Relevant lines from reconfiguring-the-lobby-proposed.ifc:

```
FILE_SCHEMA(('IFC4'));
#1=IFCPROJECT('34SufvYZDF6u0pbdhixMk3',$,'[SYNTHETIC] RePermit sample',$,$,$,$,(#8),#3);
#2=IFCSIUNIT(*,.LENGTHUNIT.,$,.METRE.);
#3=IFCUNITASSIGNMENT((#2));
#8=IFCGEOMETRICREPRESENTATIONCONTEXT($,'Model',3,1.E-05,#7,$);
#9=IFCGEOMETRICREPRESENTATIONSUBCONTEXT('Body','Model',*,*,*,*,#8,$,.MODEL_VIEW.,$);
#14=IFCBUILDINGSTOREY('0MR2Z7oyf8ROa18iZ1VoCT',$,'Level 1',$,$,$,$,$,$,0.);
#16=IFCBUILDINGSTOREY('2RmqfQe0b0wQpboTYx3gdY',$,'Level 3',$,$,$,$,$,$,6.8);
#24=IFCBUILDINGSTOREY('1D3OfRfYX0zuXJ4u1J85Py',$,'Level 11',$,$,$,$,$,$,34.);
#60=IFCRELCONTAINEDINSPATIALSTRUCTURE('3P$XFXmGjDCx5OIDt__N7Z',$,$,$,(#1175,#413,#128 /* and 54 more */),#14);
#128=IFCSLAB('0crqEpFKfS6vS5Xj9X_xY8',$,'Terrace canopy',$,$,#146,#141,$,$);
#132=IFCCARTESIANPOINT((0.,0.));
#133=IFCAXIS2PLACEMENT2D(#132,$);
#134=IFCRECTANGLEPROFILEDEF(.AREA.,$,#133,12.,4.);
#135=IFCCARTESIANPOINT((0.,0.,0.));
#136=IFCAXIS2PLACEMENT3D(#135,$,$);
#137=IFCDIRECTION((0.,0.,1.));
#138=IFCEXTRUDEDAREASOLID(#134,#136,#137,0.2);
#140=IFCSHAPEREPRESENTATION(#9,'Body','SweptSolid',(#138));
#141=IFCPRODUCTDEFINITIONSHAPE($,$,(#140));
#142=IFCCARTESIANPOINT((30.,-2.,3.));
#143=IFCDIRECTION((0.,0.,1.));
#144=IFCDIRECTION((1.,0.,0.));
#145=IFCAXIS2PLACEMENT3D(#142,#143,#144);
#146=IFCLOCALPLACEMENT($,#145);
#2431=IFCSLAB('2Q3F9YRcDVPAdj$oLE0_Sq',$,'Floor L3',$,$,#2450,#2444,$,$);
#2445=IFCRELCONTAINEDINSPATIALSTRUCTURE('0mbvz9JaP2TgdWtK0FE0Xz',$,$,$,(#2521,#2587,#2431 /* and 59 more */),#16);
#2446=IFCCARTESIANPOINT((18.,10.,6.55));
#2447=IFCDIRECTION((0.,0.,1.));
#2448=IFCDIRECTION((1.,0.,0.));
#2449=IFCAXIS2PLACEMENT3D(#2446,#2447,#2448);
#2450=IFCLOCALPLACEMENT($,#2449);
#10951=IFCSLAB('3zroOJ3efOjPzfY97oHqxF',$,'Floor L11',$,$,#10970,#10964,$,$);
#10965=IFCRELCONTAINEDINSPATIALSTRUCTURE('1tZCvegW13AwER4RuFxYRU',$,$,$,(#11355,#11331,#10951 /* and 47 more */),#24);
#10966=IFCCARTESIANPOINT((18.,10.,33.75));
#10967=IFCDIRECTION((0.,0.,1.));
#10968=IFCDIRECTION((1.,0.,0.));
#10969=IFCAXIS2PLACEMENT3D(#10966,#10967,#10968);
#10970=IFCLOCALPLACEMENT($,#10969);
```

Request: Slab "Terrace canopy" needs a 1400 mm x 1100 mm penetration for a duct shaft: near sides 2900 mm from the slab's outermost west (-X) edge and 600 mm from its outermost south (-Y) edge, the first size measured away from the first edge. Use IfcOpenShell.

```python
import numpy as np
import ifcopenshell
import ifcopenshell.api.feature
import ifcopenshell.api.geometry
import ifcopenshell.api.root
import ifcopenshell.geom
import ifcopenshell.util.placement
import ifcopenshell.util.representation
import ifcopenshell.util.shape
import ifcopenshell.util.unit

model = ifcopenshell.open("reconfiguring-the-lobby-proposed.ifc")
unit_scale = ifcopenshell.util.unit.calculate_unit_scale(model)
settings = ifcopenshell.geom.settings()


def volume(element):
    """Net volume in cubic metres, openings subtracted."""
    shape = ifcopenshell.geom.create_shape(settings, element)
    return ifcopenshell.util.shape.get_volume(shape.geometry)


slab = model.by_guid("0crqEpFKfS6vS5Xj9X_xY8")
before = volume(slab)

# Extent in the slab's own axes, in metres. The edges named are its -X and -Y sides.
slab_shape = ifcopenshell.geom.create_shape(settings, slab)
vertices = ifcopenshell.util.shape.get_vertices(slab_shape.geometry)
x_min, y_min, bottom = vertices.min(axis=0)
top = vertices[:, 2].max()

opening = ifcopenshell.api.root.create_entity(model, ifc_class="IfcOpeningElement", name="Duct shaft opening", predefined_type="OPENING")
context = ifcopenshell.util.representation.get_context(model, "Model", "Body", "MODEL_VIEW")
width, depth = 1.4, 1.1
outline = [(0.0, 0.0), (width, 0.0), (width, depth), (0.0, depth), (0.0, 0.0)]
# Overshoot both faces by 50 mm so the cut is clean.
shape = ifcopenshell.api.geometry.add_slab_representation(
    model, context=context, depth=top - bottom + 0.1, polyline=outline
)
ifcopenshell.api.geometry.assign_representation(model, product=opening, representation=shape)

matrix = ifcopenshell.util.placement.get_local_placement(slab.ObjectPlacement)
matrix[:, 3] = matrix @ np.append(np.array([x_min + 2.9, y_min + 0.6, bottom - 0.05]) / unit_scale, 1.0)
ifcopenshell.api.geometry.edit_object_placement(model, product=opening, matrix=matrix, is_si=False)
ifcopenshell.api.feature.add_feature(model, feature=opening, element=slab)

after = volume(slab)

print(f"slab volume {before:.3f} -> {after:.3f} m3")

model.write("reconfiguring-the-lobby-proposed_v2.ifc")
```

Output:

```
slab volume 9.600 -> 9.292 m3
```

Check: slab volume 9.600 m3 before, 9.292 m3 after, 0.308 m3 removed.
